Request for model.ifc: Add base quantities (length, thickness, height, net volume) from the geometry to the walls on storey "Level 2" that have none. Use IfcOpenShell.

First a look at what the model holds.

```python
import ifcopenshell
import ifcopenshell.util.element
import ifcopenshell.util.unit

model = ifcopenshell.open("model.ifc")
print(model.schema)
for unit_type in ("LENGTHUNIT", "AREAUNIT", "VOLUMEUNIT"):
    print(unit_type, ifcopenshell.util.unit.calculate_unit_scale(model, unit_type))
storey = next(s for s in model.by_type("IfcBuildingStorey") if s.Name == "Level 2")
walls = [e for e in ifcopenshell.util.element.get_decomposition(storey) if e.is_a("IfcWall")]
for e in sorted(walls, key=lambda e: e.id()):
    print(e.id(), e.is_a(), e.Name, list(ifcopenshell.util.element.get_psets(e, qtos_only=True)), sep=" | ")
```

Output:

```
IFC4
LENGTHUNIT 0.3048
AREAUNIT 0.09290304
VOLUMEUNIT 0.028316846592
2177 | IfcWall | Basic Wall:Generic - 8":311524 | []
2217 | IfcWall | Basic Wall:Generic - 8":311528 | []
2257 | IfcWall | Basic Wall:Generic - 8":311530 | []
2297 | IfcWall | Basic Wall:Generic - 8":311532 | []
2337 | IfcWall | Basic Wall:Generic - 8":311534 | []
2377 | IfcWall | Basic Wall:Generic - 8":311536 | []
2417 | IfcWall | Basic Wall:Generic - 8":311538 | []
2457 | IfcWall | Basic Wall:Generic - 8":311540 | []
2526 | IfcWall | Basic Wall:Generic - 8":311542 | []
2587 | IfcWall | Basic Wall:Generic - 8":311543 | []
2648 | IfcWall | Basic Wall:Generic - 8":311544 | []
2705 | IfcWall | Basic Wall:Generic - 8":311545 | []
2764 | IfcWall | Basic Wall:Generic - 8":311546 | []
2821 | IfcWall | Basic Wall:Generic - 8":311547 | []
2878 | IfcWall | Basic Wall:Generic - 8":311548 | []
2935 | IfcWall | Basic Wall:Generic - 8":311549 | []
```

```python
import ifcopenshell
import ifcopenshell.api.pset
import ifcopenshell.geom
import ifcopenshell.util.element
import ifcopenshell.util.shape
import ifcopenshell.util.unit

model = ifcopenshell.open("model.ifc")
unit_scale = ifcopenshell.util.unit.calculate_unit_scale(model)
volume_scale = ifcopenshell.util.unit.calculate_unit_scale(model, "VOLUMEUNIT")
settings = ifcopenshell.geom.settings()

storey = next(s for s in model.by_type("IfcBuildingStorey") if s.Name == "Level 2")
walls = [e for e in ifcopenshell.util.element.get_decomposition(storey) if e.is_a("IfcWall")]

for e in sorted(walls, key=lambda e: e.id()):
    if ifcopenshell.util.element.get_psets(e, qtos_only=True, should_inherit=False):
        continue
    # Geometry comes back in metres, in the element's own axes.
    shape = ifcopenshell.geom.create_shape(settings, e)
    values = {
        "Length": ifcopenshell.util.shape.get_x(shape.geometry) / unit_scale,
        "Width": ifcopenshell.util.shape.get_y(shape.geometry) / unit_scale,
        "Height": ifcopenshell.util.shape.get_z(shape.geometry) / unit_scale,
        "NetVolume": ifcopenshell.util.shape.get_volume(shape.geometry) / volume_scale,
    }
    qto = ifcopenshell.api.pset.add_qto(model, product=e, name="Qto_WallBaseQuantities")
    ifcopenshell.api.pset.edit_qto(model, qto=qto, properties=values)
    print(e.id(), {k: round(v, 3) for k, v in values.items()})

model.write("model-out.ifc")
```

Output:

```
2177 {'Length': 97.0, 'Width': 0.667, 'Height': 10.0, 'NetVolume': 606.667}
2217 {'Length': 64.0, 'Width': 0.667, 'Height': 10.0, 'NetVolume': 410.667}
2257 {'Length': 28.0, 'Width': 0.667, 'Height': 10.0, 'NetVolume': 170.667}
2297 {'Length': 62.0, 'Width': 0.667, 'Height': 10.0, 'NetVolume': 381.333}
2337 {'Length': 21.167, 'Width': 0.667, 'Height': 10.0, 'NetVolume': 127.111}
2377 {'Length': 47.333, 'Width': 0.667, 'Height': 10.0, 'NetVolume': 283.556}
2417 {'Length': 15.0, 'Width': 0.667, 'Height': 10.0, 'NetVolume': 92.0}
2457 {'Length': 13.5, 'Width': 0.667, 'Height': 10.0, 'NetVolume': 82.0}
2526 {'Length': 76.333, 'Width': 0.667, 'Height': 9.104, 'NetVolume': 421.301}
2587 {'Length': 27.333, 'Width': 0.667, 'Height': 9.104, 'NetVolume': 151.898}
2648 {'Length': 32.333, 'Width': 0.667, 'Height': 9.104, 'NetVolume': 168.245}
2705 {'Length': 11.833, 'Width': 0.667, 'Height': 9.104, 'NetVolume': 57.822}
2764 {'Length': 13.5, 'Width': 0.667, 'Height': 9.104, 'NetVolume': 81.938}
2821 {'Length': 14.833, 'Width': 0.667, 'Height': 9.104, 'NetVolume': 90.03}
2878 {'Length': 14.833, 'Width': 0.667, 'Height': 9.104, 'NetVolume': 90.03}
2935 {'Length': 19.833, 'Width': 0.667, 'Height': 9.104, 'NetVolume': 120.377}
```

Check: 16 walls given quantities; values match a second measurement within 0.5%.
